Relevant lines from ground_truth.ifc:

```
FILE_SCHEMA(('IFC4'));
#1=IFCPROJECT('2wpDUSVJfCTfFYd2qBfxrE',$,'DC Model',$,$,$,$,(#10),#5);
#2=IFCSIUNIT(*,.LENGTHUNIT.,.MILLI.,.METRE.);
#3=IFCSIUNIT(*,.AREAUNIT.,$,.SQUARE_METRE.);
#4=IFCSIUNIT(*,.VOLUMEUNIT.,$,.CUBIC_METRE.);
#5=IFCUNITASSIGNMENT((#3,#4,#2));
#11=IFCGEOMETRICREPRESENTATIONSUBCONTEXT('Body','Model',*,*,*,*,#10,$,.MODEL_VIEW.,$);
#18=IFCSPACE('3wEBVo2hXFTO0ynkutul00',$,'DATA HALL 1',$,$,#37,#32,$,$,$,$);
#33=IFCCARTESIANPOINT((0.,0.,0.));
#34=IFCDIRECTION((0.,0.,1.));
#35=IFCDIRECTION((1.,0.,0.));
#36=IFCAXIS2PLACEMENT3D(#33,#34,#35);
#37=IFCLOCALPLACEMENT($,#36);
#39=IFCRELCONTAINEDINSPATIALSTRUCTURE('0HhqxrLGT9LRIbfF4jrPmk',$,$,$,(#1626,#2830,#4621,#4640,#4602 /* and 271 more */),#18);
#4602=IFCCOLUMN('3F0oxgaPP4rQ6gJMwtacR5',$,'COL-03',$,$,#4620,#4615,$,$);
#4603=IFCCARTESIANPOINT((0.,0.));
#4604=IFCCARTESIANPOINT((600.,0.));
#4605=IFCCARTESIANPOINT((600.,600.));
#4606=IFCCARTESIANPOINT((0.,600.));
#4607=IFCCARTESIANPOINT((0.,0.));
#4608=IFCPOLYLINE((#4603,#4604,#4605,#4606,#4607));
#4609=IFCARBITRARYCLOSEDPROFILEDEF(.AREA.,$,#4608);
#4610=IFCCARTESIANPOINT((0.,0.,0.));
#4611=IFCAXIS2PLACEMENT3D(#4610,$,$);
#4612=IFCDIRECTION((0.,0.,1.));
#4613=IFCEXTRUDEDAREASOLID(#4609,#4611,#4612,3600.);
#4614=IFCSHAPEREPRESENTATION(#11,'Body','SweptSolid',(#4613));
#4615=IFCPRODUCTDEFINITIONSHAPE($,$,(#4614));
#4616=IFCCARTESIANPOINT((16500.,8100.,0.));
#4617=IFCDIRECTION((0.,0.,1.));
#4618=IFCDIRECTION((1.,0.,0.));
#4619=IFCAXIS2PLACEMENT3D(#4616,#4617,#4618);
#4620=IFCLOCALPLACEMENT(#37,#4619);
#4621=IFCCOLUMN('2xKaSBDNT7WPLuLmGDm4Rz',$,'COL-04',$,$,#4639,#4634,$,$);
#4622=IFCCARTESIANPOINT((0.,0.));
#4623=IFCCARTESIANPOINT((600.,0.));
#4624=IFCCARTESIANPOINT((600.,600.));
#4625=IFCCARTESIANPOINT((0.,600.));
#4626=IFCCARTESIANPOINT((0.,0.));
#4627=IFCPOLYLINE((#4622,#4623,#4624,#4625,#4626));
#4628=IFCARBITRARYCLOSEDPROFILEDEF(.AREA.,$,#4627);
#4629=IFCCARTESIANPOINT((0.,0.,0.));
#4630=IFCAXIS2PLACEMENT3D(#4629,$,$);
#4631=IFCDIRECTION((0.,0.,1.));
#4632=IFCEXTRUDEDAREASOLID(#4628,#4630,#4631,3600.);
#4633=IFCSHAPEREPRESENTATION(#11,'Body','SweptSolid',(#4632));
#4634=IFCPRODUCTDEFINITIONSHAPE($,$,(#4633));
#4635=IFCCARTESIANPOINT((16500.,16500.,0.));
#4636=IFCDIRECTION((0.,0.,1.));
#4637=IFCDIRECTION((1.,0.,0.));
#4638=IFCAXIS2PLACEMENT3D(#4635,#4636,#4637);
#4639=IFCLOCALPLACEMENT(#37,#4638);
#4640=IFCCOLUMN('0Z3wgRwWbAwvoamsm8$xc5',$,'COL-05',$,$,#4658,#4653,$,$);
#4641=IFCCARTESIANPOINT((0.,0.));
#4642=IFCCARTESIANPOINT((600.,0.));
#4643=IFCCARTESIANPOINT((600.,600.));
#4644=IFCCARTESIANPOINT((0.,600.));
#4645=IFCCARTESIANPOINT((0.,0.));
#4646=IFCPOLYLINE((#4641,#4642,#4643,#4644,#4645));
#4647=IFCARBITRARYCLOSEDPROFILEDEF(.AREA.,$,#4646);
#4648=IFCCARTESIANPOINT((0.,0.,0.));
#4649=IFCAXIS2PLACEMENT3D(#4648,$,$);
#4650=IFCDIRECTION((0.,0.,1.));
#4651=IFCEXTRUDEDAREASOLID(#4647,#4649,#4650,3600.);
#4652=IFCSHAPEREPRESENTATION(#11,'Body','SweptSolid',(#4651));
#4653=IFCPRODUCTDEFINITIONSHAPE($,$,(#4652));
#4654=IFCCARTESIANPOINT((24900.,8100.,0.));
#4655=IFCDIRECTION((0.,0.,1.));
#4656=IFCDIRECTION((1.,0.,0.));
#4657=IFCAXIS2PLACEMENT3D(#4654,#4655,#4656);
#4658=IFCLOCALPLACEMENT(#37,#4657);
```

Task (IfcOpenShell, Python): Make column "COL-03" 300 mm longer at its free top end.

```python
import ifcopenshell
import ifcopenshell.util.representation

model = ifcopenshell.open("ground_truth.ifc")

member = model.by_guid("3F0oxgaPP4rQ6gJMwtacR5")
change = 300.0

# The extrusion runs towards the end named, so only its depth changes.
body = ifcopenshell.util.representation.get_representation(member, "Model", "Body")
solid = body.Items[0]
old_length = solid.Depth
solid.Depth += change

print(f"length {old_length:g} -> {solid.Depth:g}")

model.write("ground_truth_v2.ifc")
```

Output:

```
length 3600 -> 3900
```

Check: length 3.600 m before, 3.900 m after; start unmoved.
